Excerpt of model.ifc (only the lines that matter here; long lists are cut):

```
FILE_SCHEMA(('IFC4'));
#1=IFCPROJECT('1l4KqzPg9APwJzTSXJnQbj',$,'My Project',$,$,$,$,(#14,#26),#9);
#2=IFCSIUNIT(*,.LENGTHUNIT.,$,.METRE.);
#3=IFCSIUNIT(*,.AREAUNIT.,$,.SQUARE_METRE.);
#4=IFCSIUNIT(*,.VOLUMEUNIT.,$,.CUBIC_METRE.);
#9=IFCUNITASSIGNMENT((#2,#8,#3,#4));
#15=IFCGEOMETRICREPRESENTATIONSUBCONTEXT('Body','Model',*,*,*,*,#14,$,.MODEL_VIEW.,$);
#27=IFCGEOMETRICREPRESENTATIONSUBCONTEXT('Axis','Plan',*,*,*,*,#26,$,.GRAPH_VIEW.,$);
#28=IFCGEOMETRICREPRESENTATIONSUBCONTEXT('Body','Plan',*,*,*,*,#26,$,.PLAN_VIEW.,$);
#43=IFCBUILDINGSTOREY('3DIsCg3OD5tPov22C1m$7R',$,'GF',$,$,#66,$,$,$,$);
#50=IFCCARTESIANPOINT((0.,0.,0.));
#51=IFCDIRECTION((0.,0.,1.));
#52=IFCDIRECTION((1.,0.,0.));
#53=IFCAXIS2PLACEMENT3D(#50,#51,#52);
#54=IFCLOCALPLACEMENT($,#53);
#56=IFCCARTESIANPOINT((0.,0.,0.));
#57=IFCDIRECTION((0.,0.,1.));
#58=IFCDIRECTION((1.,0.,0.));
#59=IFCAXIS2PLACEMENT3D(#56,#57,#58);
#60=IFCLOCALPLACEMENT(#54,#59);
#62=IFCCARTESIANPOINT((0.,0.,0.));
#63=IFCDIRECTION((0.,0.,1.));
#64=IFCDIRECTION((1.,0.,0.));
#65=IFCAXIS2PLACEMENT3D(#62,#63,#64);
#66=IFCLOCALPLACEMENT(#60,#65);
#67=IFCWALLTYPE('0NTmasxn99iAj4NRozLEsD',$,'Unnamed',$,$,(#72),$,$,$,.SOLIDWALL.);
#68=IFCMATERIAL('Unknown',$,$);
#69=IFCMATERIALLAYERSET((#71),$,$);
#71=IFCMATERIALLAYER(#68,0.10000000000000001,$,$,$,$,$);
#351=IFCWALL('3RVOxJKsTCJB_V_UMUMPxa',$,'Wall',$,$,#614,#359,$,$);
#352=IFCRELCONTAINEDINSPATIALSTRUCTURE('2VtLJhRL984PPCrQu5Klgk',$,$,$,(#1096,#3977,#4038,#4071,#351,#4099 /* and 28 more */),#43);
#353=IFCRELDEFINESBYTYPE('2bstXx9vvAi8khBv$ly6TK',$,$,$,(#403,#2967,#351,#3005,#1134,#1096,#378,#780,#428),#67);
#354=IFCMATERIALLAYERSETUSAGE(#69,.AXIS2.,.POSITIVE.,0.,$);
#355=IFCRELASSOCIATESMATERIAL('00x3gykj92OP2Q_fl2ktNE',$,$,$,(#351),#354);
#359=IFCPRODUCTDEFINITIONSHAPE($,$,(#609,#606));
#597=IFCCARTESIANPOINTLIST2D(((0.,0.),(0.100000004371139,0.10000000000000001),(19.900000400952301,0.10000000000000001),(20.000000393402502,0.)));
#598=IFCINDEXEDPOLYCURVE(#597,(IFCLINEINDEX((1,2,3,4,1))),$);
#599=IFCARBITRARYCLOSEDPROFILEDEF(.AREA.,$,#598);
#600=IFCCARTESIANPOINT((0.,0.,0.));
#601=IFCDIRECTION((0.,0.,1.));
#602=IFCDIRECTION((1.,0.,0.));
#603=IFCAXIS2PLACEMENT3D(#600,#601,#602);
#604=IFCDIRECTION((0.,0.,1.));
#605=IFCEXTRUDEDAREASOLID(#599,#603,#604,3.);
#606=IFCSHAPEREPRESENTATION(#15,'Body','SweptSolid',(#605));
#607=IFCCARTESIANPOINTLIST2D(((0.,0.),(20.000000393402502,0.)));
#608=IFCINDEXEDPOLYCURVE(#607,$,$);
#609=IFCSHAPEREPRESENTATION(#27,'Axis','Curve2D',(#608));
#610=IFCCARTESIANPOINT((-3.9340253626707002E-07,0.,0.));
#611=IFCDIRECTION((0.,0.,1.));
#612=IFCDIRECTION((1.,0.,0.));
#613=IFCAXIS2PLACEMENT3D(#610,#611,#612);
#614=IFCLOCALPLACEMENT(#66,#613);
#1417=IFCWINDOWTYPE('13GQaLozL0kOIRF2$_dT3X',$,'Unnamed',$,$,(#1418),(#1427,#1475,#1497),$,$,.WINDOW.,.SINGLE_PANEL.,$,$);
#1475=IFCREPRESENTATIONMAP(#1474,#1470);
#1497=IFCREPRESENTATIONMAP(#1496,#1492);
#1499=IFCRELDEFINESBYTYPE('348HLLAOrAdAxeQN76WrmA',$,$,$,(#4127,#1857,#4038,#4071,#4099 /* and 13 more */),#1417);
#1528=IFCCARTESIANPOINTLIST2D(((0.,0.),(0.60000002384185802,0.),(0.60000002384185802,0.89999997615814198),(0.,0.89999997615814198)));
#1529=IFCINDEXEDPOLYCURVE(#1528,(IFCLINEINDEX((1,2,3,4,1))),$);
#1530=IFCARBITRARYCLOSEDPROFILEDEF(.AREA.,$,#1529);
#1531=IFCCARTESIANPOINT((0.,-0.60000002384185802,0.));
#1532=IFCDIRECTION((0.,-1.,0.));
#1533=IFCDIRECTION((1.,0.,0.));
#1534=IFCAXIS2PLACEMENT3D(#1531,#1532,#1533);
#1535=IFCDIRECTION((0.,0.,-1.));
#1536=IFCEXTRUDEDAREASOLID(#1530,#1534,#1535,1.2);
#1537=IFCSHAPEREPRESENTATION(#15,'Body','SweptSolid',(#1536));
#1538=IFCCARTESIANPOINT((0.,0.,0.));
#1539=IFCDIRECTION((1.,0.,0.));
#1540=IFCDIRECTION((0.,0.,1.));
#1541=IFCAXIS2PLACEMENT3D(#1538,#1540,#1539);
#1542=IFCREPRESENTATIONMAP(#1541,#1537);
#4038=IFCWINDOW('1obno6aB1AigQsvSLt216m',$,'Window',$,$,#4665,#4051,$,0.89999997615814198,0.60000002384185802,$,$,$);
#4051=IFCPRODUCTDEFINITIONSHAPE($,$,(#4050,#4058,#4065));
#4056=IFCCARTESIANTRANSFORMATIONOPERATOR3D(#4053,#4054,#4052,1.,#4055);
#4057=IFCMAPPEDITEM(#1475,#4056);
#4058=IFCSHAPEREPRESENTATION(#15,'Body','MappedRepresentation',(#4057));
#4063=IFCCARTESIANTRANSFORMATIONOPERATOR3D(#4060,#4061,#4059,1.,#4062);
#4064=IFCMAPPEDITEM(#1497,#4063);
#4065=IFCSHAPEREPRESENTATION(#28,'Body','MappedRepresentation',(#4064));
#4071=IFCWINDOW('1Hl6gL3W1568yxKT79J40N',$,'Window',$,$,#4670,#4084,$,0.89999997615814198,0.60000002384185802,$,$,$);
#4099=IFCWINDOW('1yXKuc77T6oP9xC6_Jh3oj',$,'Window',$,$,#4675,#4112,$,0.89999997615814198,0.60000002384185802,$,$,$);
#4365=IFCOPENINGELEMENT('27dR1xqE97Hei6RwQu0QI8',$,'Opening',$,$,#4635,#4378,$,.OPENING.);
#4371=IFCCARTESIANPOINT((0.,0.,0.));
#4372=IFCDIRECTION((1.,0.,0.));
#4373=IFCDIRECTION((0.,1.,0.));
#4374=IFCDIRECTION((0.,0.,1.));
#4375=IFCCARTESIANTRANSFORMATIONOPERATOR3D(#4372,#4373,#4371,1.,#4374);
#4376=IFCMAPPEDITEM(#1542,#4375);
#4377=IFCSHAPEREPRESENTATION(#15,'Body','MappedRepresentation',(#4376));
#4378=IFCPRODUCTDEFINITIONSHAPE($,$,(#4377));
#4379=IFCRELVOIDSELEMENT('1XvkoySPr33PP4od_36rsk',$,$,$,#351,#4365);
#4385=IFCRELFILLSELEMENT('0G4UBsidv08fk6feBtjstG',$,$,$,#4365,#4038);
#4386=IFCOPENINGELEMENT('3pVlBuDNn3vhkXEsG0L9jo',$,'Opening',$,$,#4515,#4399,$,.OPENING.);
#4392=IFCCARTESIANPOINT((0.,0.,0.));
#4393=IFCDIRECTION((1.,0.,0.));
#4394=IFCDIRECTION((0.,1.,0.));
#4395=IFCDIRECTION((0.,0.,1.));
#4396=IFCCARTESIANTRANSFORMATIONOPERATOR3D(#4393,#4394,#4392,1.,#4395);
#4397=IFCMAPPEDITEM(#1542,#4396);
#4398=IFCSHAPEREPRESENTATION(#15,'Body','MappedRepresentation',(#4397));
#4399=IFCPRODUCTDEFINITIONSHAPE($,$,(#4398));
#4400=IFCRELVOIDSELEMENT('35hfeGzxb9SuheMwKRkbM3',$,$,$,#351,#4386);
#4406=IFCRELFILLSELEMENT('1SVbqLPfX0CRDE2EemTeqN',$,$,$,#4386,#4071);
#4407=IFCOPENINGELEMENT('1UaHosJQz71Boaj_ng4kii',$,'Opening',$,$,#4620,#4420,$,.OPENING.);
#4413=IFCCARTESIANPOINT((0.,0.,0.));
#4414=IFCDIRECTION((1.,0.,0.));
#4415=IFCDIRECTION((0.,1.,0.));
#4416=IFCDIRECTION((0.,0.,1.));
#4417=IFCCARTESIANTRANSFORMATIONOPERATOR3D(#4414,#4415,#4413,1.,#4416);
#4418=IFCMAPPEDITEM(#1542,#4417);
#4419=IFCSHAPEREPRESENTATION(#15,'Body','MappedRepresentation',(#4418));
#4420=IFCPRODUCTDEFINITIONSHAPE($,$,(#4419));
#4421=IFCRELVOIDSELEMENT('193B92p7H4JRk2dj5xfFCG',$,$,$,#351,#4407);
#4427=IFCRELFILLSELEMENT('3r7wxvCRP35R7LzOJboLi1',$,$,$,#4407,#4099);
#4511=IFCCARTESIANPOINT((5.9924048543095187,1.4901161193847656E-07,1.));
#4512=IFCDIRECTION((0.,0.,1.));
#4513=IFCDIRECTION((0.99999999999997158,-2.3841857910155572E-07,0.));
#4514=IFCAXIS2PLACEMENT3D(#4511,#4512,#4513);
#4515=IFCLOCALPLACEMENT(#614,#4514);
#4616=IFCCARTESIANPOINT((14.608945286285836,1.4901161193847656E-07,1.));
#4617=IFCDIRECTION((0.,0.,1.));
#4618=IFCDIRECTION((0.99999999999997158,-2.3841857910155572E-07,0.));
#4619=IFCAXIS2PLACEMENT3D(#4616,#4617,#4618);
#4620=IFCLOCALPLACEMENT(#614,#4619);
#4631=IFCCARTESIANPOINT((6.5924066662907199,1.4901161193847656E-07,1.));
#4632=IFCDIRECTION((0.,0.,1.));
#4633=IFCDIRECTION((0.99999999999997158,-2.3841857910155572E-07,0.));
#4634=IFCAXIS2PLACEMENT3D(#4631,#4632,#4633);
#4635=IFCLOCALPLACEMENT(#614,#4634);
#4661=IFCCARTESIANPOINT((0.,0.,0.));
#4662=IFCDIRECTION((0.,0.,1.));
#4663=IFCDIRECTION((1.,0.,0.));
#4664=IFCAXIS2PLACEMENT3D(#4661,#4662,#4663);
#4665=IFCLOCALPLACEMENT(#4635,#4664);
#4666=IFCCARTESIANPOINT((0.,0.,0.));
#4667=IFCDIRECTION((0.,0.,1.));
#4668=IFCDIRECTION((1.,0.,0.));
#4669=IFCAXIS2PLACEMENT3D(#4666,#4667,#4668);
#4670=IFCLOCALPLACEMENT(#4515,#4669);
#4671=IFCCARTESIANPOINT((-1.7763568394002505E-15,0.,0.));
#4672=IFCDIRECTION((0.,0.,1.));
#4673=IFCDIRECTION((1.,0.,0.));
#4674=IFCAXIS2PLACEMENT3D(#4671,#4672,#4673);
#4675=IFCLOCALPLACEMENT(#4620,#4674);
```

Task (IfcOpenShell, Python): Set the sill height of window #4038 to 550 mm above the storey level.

```python
import numpy as np
import ifcopenshell
import ifcopenshell.api.geometry
import ifcopenshell.geom
import ifcopenshell.util.element
import ifcopenshell.util.placement
import ifcopenshell.util.shape
import ifcopenshell.util.unit

model = ifcopenshell.open("model.ifc")
unit_scale = ifcopenshell.util.unit.calculate_unit_scale(model)

window = model.by_guid("1obno6aB1AigQsvSLt216m")
opening = window.FillsVoids[0].RelatingOpeningElement
storey = ifcopenshell.util.element.get_container(window, ifc_class="IfcBuildingStorey")
level = ifcopenshell.util.placement.get_local_placement(storey.ObjectPlacement)[2, 3]

# The opening's origin need not be at the sill, so measure its lowest point.
shape = ifcopenshell.geom.create_shape(ifcopenshell.geom.settings(), opening)
bottom = ifcopenshell.util.shape.get_shape_bottom_elevation(shape, shape.geometry) / unit_scale
dz = level + 0.55 - bottom

shift = np.array([0.0, 0.0, dz])
# The window is placed relative to its opening, so it follows when the opening moves.
matrix = ifcopenshell.util.placement.get_local_placement(opening.ObjectPlacement)
matrix[:3, 3] += shift
ifcopenshell.api.geometry.edit_object_placement(
    model, product=opening, matrix=matrix, is_si=False, should_transform_children=True
)

print(f"moved by {dz * unit_scale:+.3f} m")

model.write("model_updated.ifc")
```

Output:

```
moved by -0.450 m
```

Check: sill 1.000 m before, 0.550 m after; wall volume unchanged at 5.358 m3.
